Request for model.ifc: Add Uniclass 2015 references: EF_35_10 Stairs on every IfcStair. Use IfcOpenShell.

First a look at what the model holds.

```python
import ifcopenshell

model = ifcopenshell.open("model.ifc")
print(model.schema)
print("classifications:", [c.Name for c in model.by_type("IfcClassification")])
for ifc_class in ("IfcDoor", "IfcRoof", "IfcStair", "IfcWall", "IfcWindow"):
    print(ifc_class, len(model.by_type(ifc_class)))
```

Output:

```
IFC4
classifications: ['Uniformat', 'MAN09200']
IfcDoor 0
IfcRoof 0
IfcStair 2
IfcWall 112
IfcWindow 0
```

```python
import ifcopenshell
import ifcopenshell.api.classification

model = ifcopenshell.open("model.ifc")

system = ifcopenshell.api.classification.add_classification(model, classification="Uniclass 2015")

codes = {
    "IfcStair": ("EF_35_10", "Stairs"),
}
for ifc_class, (code, name) in codes.items():
    products = model.by_type(ifc_class)
    ifcopenshell.api.classification.add_reference(
        model, products=products, classification=system, identification=code, name=name
    )
    print(code, len(products))

model.write("model_rev.ifc")
```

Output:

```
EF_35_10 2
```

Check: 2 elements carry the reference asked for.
